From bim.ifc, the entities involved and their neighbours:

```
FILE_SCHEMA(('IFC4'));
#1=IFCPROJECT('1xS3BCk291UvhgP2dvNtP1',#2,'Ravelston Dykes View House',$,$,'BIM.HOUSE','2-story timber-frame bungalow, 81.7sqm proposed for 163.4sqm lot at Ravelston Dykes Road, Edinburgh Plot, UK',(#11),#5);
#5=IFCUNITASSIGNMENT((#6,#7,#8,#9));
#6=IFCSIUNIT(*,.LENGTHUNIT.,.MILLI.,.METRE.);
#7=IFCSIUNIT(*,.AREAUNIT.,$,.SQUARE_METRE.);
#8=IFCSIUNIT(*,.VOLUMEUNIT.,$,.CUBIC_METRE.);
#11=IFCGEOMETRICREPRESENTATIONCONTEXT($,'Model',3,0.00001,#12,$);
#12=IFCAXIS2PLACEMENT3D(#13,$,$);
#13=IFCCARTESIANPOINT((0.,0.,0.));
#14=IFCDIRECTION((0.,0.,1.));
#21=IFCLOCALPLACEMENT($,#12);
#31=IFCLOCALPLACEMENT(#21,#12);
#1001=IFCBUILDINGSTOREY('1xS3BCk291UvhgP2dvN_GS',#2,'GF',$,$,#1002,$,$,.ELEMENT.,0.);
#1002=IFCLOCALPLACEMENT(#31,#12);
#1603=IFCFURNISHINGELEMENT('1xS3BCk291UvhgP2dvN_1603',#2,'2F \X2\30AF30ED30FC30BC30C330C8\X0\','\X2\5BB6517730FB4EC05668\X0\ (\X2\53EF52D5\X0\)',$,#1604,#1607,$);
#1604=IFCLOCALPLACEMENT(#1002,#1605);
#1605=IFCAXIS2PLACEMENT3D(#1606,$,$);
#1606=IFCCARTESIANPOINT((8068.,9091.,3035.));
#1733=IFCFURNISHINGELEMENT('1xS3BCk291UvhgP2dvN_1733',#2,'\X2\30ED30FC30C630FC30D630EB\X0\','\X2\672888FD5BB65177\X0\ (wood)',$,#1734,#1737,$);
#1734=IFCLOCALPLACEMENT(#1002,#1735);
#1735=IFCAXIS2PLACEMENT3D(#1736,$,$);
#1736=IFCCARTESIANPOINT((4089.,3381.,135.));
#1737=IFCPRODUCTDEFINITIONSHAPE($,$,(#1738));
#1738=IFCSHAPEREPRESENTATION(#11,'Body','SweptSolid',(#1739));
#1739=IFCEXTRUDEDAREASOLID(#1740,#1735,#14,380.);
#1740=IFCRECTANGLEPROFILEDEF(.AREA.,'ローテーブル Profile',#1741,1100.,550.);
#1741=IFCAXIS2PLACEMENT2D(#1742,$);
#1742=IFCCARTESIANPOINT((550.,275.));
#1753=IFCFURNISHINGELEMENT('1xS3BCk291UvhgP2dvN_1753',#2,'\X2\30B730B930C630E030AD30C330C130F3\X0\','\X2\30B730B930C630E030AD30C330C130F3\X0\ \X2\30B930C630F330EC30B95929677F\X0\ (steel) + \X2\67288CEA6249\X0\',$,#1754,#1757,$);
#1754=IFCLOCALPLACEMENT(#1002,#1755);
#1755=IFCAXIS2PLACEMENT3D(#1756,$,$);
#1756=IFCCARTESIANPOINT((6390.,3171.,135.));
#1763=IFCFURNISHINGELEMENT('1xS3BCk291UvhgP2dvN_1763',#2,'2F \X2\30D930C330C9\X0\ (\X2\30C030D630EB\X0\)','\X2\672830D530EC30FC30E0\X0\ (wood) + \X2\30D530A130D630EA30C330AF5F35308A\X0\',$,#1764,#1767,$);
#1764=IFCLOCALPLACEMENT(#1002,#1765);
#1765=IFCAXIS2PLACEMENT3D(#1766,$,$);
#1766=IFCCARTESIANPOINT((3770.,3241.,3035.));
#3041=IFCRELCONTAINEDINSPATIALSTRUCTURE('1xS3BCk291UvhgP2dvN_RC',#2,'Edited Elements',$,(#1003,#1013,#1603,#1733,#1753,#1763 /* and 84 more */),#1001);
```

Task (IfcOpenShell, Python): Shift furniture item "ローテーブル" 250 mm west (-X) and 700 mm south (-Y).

```python
import ifcopenshell
import ifcopenshell.api.geometry
import ifcopenshell.util.placement
import ifcopenshell.util.unit

model = ifcopenshell.open("bim.ifc")
unit_scale = ifcopenshell.util.unit.calculate_unit_scale(model)

item = model.by_id(1733)
matrix = ifcopenshell.util.placement.get_local_placement(item.ObjectPlacement)
matrix[0, 3] -= 0.25 / unit_scale
matrix[1, 3] -= 0.7 / unit_scale
ifcopenshell.api.geometry.edit_object_placement(model, product=item, matrix=matrix, is_si=False)

print(ifcopenshell.util.placement.get_local_placement(item.ObjectPlacement).round(3) + 0.0)

model.write("bim_edited.ifc")
```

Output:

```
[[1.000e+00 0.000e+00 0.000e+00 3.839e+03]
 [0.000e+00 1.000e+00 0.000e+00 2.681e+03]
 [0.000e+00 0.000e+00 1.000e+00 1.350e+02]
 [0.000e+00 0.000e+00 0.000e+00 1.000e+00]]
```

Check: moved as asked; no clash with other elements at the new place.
